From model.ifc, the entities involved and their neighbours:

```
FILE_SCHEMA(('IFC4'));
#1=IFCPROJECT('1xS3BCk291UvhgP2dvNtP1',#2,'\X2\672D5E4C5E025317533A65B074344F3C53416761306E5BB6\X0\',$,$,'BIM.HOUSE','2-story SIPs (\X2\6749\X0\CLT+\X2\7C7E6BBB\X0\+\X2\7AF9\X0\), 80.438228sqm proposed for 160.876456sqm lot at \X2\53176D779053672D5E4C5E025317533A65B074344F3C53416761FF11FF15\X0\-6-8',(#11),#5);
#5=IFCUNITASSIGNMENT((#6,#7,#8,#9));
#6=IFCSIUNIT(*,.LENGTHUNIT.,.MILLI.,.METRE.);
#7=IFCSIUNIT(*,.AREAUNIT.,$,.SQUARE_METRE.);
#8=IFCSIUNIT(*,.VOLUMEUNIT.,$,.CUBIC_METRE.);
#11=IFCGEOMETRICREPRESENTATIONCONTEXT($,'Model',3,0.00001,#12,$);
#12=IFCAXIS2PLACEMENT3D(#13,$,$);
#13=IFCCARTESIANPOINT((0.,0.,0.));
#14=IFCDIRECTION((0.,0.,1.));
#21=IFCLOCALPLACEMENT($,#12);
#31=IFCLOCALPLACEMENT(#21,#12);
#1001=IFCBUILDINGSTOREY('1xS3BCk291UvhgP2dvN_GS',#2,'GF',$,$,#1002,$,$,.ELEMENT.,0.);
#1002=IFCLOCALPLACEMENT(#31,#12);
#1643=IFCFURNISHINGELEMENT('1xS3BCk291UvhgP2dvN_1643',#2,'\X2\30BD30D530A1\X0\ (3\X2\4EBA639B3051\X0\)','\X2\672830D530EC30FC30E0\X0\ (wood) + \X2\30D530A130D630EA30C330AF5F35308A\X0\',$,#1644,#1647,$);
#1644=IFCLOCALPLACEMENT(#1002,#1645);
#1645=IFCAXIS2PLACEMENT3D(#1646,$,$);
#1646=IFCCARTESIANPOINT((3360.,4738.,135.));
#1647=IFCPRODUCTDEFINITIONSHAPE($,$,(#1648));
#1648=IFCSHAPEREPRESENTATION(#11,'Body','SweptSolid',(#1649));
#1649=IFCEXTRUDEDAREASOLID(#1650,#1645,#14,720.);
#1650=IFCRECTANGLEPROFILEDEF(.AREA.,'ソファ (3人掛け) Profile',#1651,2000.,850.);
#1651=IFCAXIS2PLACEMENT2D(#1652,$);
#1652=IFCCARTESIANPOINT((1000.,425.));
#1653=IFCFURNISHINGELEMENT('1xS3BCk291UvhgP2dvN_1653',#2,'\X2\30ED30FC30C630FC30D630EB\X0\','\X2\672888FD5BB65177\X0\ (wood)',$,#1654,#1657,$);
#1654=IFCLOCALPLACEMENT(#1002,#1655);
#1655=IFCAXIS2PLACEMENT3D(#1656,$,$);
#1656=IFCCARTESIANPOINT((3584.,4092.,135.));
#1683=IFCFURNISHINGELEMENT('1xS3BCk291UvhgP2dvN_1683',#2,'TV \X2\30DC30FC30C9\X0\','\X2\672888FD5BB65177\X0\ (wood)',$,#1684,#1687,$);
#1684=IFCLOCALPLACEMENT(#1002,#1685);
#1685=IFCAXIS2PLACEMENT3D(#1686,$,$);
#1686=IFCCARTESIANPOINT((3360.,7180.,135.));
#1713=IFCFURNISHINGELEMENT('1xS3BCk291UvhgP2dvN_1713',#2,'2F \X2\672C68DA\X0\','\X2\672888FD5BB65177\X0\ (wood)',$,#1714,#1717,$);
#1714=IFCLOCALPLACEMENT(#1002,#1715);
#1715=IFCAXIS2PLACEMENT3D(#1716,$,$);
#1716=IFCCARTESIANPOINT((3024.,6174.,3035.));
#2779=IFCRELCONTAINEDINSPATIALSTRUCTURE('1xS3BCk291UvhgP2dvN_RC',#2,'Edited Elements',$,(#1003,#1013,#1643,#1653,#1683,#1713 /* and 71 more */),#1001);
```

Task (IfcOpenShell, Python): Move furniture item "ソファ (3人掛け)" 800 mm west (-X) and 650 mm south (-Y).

```python
import ifcopenshell
import ifcopenshell.api.geometry
import ifcopenshell.util.placement

model = ifcopenshell.open("model.ifc")

item = model.by_guid("1xS3BCk291UvhgP2dvN_1643")
matrix = ifcopenshell.util.placement.get_local_placement(item.ObjectPlacement)
matrix[0, 3] -= 800.0
matrix[1, 3] -= 650.0
ifcopenshell.api.geometry.edit_object_placement(model, product=item, matrix=matrix, is_si=False)

print(ifcopenshell.util.placement.get_local_placement(item.ObjectPlacement).round(3) + 0.0)

model.write("model_edited.ifc")
```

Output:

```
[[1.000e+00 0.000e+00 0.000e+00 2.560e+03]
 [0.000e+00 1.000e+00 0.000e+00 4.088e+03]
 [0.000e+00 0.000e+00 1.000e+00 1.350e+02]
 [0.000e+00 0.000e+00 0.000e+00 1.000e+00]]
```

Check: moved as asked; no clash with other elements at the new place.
